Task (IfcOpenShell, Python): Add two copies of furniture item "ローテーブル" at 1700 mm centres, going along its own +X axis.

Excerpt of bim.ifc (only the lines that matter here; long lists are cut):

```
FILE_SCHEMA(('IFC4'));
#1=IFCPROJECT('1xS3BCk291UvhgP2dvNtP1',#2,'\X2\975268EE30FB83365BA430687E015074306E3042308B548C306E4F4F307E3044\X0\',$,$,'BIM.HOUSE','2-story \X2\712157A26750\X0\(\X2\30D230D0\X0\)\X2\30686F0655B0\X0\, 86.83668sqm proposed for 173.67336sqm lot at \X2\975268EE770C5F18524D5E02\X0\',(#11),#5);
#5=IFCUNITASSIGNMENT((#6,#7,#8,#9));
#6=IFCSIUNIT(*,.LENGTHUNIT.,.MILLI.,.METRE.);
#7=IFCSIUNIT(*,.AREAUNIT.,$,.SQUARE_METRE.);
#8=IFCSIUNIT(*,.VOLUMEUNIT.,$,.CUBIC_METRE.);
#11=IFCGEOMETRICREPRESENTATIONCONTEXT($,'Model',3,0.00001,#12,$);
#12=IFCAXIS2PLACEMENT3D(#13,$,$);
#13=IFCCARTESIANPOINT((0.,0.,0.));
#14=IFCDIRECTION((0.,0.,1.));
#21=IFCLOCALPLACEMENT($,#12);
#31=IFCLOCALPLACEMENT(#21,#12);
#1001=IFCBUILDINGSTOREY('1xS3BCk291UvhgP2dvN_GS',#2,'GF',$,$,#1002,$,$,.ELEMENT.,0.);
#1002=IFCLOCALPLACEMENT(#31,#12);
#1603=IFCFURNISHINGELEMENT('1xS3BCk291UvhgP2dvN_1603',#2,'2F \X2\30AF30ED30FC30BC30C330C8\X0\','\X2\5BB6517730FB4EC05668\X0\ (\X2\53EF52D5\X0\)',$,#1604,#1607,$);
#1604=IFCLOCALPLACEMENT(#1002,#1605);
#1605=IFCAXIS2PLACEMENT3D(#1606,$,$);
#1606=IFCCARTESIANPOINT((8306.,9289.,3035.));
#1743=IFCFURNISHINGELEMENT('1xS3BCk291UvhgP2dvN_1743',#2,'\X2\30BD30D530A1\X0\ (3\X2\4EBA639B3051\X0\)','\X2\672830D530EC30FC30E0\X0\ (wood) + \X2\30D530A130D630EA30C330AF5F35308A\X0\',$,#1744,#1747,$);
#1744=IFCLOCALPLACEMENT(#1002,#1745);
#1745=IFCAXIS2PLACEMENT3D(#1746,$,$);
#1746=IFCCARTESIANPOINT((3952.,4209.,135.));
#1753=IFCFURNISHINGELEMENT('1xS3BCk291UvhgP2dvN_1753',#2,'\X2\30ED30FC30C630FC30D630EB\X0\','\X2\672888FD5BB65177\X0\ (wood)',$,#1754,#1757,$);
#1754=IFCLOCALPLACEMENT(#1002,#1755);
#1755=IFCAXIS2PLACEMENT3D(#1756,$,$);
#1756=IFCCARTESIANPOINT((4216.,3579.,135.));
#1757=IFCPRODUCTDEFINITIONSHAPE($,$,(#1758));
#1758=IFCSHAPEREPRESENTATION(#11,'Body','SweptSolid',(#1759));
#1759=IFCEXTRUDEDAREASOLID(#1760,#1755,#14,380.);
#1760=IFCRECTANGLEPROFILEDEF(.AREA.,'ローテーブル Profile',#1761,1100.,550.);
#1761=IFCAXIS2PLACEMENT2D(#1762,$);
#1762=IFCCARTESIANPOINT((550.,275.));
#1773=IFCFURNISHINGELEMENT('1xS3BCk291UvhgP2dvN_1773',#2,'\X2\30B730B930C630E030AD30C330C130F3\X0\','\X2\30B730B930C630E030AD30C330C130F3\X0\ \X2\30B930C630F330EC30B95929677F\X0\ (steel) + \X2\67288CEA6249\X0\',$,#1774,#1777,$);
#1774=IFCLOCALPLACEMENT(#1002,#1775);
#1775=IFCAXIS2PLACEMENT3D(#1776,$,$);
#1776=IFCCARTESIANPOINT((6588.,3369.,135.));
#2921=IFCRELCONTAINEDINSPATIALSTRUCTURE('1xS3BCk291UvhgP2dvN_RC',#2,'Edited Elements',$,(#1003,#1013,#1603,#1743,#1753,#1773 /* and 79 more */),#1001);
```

```python
import ifcopenshell
import ifcopenshell.api.geometry
import ifcopenshell.api.root
import ifcopenshell.util.element
import ifcopenshell.util.placement

model = ifcopenshell.open("bim.ifc")


def reuse_history(source, copy):
    """copy_class also copies each property set's owner history, people and application; keep the originals."""
    for rel in copy.IsDefinedBy:
        if rel.is_a("IfcRelDefinesByProperties") and (history := rel.RelatingPropertyDefinition.OwnerHistory):
            rel.RelatingPropertyDefinition.OwnerHistory = source.OwnerHistory
            ifcopenshell.util.element.remove_deep2(model, history)


source = model.by_guid("1xS3BCk291UvhgP2dvN_1753")
base = ifcopenshell.util.placement.get_local_placement(source.ObjectPlacement)
step = base[:3, 0] * 1700.0

for i in range(1, 3):
    copy = ifcopenshell.api.root.copy_class(model, product=source)
    copy.Representation = ifcopenshell.util.element.copy_deep(
        model, source.Representation, exclude=["IfcGeometricRepresentationContext", "IfcRepresentationMap"]
    )
    reuse_history(source, copy)
    matrix = base.copy()
    matrix[:3, 3] += i * step
    print("added at", matrix[:3, 3].round(3) + 0.0)
    ifcopenshell.api.geometry.edit_object_placement(model, product=copy, matrix=matrix, is_si=False)

model.write("bim_updated.ifc")
```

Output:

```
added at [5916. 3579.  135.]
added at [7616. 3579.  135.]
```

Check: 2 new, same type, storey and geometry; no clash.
